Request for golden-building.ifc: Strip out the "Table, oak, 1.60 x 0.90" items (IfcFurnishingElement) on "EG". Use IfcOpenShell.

First a look at what the model holds.

```python
import ifcopenshell
import ifcopenshell.util.element

model = ifcopenshell.open("golden-building.ifc")
print(model.schema)
storey = next(s for s in model.by_type("IfcBuildingStorey") if s.Name == "EG")
furniture = [e for e in ifcopenshell.util.element.get_decomposition(storey) if e.is_a("IfcFurnishingElement")]
seen = {}
for e in furniture:
    element_type = ifcopenshell.util.element.get_type(e)
    name = element_type.Name if element_type not in (None, e) else None
    seen[name] = seen.get(name, 0) + 1
for name, count in sorted(seen.items(), key=str):
    print(count, "x", name)
```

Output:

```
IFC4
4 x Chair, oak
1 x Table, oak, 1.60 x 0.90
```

```python
import ifcopenshell
import ifcopenshell.api.root
import ifcopenshell.util.element

model = ifcopenshell.open("golden-building.ifc")

storey = next(s for s in model.by_type("IfcBuildingStorey") if s.Name == "EG")
furniture = [e for e in ifcopenshell.util.element.get_decomposition(storey) if e.is_a("IfcFurnishingElement")]
targets = [e for e in furniture if (t := ifcopenshell.util.element.get_type(e)) not in (None, e) and t.Name == "Table, oak, 1.60 x 0.90"]

for e in targets:
    ifcopenshell.api.root.remove_product(model, product=e)
print(len(targets), "removed")

model.write("golden-building_edited.ifc")
```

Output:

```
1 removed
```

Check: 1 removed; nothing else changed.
